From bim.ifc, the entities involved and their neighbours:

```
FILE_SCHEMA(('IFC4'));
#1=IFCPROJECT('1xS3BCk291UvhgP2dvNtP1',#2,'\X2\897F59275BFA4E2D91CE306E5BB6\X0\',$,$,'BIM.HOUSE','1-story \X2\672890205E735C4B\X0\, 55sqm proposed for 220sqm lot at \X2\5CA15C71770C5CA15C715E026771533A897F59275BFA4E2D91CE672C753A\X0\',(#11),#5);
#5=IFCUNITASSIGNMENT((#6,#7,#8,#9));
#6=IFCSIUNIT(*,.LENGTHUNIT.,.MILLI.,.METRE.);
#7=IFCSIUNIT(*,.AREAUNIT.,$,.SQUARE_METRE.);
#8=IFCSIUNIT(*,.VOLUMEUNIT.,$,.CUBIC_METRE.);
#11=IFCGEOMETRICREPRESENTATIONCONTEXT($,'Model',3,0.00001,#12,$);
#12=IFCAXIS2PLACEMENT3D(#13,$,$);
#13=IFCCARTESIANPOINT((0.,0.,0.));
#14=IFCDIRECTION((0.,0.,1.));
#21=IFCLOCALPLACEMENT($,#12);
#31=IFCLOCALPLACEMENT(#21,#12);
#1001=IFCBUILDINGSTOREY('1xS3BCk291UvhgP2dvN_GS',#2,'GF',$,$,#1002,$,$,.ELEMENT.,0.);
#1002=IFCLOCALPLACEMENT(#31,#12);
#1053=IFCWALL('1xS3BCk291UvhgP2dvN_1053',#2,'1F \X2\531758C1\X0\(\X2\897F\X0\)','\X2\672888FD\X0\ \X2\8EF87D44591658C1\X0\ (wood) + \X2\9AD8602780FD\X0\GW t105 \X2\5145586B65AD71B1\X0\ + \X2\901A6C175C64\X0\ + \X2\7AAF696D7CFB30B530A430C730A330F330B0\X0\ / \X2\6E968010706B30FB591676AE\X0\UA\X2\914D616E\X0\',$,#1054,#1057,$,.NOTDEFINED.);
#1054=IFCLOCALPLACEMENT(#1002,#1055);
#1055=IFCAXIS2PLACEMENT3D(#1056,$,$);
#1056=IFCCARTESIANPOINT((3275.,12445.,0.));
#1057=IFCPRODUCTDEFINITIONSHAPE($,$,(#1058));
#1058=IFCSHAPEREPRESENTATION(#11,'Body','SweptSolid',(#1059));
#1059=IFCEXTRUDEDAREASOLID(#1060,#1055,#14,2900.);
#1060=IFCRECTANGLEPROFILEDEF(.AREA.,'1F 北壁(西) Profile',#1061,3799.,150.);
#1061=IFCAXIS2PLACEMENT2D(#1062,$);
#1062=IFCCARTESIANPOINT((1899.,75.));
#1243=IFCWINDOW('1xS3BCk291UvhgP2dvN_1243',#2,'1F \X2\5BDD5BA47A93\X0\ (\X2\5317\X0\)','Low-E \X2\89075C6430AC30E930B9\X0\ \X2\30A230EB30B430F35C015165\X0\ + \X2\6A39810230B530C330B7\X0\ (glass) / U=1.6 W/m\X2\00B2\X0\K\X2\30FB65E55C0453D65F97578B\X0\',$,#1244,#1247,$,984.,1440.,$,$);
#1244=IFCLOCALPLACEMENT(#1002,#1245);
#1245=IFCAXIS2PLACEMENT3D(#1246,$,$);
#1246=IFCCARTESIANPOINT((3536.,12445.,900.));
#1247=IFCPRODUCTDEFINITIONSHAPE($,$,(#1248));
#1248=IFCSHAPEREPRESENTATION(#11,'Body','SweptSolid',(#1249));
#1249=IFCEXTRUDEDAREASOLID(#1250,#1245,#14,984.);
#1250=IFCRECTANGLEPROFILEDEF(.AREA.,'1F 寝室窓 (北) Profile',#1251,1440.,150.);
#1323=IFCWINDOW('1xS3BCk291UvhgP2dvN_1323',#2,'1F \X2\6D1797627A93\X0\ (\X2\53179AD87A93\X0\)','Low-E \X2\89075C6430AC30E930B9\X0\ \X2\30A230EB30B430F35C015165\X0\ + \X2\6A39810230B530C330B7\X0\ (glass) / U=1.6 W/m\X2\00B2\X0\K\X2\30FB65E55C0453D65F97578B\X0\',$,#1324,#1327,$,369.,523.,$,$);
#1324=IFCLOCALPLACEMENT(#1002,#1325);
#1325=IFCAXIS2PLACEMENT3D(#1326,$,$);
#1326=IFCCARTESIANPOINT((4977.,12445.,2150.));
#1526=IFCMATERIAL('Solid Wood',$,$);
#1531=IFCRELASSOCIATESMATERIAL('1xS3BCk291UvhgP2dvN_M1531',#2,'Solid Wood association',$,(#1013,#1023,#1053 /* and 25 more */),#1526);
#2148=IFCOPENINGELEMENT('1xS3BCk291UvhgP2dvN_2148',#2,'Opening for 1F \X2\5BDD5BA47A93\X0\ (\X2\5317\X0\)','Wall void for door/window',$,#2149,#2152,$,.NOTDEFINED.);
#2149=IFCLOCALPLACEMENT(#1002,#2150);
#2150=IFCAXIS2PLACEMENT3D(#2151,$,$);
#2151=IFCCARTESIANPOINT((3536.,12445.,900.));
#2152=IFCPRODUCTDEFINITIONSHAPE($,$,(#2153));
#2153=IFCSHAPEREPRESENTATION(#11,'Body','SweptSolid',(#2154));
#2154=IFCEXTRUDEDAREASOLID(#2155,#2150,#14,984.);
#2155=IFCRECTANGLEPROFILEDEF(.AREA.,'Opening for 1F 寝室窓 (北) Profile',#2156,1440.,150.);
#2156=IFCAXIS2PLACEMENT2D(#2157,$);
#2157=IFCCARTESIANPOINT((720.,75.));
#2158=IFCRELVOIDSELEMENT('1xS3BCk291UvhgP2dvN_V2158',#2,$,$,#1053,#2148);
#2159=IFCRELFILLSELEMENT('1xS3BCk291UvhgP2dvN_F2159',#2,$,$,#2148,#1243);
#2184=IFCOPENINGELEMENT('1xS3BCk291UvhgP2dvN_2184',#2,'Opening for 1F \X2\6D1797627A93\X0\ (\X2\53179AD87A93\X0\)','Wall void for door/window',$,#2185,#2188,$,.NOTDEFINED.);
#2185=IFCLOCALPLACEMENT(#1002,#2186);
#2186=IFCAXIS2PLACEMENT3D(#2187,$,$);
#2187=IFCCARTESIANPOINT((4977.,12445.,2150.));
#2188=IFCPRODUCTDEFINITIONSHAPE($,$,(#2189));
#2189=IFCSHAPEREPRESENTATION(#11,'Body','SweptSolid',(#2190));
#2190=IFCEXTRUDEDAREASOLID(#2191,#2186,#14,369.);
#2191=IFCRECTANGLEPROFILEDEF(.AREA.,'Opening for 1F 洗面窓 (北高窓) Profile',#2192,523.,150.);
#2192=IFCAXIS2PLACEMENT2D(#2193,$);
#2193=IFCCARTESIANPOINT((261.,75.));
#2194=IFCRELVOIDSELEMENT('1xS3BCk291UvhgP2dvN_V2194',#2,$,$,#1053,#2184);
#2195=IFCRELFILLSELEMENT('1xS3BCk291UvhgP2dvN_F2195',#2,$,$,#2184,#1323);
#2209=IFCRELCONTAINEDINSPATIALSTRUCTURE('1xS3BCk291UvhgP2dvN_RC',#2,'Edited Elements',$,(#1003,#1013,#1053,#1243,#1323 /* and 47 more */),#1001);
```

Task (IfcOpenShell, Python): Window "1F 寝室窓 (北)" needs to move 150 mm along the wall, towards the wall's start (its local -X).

```python
import ifcopenshell
import ifcopenshell.api.geometry
import ifcopenshell.util.placement

model = ifcopenshell.open("bim.ifc")

window = model.by_guid("1xS3BCk291UvhgP2dvN_1243")
opening = window.FillsVoids[0].RelatingOpeningElement
wall = opening.VoidsElements[0].RelatingBuildingElement

wall_matrix = ifcopenshell.util.placement.get_local_placement(wall.ObjectPlacement)
shift = wall_matrix[:3, 0] * -150.0
before = ifcopenshell.util.placement.get_local_placement(window.ObjectPlacement)[:3, 3].copy()

# The window is not placed relative to its opening, so move both.
for product in (opening, window):
    matrix = ifcopenshell.util.placement.get_local_placement(product.ObjectPlacement)
    matrix[:3, 3] += shift
    ifcopenshell.api.geometry.edit_object_placement(model, product=product, matrix=matrix, is_si=False)

after = ifcopenshell.util.placement.get_local_placement(window.ObjectPlacement)[:3, 3]
print("window moved by", (after - before).round(3) + 0.0)

model.write("bim_v2.ifc")
```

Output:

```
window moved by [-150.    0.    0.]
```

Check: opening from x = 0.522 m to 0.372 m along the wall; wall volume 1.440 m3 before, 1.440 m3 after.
